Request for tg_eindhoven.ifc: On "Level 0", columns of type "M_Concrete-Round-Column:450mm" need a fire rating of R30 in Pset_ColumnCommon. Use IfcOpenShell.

First a look at what the model holds.

```python
import ifcopenshell
import ifcopenshell.util.element

model = ifcopenshell.open("tg_eindhoven.ifc")
print(model.schema)
storey = next(s for s in model.by_type("IfcBuildingStorey") if s.Name == "Level 0")
columns = [e for e in ifcopenshell.util.element.get_decomposition(storey) if e.is_a("IfcColumn")]
seen = {}
for e in columns:
    element_type = ifcopenshell.util.element.get_type(e)
    key = (element_type.Name if element_type != e and element_type else None, ifcopenshell.util.element.get_pset(e, "Pset_ColumnCommon", "FireRating"))
    seen[key] = seen.get(key, 0) + 1
for (name, value), count in sorted(seen.items(), key=str):
    print(count, "x", name, "|", value)
```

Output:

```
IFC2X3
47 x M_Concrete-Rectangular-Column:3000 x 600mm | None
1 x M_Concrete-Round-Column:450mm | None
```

```python
import ifcopenshell
import ifcopenshell.api.pset
import ifcopenshell.util.element

model = ifcopenshell.open("tg_eindhoven.ifc")

storey = next(s for s in model.by_type("IfcBuildingStorey") if s.Name == "Level 0")
columns = [e for e in ifcopenshell.util.element.get_decomposition(storey) if e.is_a("IfcColumn")]

count = 0
for e in columns:
    element_type = ifcopenshell.util.element.get_type(e)
    if element_type in (None, e) or element_type.Name != "M_Concrete-Round-Column:450mm":
        continue
    # add_pset returns the element's existing set when there is one.
    pset = ifcopenshell.api.pset.add_pset(model, product=e, name="Pset_ColumnCommon")
    ifcopenshell.api.pset.edit_pset(model, pset=pset, properties={"FireRating": "R30"})
    count += 1

print(count, "columns updated")

model.write("tg_eindhoven_edited.ifc")
```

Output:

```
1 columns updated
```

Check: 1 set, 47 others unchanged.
